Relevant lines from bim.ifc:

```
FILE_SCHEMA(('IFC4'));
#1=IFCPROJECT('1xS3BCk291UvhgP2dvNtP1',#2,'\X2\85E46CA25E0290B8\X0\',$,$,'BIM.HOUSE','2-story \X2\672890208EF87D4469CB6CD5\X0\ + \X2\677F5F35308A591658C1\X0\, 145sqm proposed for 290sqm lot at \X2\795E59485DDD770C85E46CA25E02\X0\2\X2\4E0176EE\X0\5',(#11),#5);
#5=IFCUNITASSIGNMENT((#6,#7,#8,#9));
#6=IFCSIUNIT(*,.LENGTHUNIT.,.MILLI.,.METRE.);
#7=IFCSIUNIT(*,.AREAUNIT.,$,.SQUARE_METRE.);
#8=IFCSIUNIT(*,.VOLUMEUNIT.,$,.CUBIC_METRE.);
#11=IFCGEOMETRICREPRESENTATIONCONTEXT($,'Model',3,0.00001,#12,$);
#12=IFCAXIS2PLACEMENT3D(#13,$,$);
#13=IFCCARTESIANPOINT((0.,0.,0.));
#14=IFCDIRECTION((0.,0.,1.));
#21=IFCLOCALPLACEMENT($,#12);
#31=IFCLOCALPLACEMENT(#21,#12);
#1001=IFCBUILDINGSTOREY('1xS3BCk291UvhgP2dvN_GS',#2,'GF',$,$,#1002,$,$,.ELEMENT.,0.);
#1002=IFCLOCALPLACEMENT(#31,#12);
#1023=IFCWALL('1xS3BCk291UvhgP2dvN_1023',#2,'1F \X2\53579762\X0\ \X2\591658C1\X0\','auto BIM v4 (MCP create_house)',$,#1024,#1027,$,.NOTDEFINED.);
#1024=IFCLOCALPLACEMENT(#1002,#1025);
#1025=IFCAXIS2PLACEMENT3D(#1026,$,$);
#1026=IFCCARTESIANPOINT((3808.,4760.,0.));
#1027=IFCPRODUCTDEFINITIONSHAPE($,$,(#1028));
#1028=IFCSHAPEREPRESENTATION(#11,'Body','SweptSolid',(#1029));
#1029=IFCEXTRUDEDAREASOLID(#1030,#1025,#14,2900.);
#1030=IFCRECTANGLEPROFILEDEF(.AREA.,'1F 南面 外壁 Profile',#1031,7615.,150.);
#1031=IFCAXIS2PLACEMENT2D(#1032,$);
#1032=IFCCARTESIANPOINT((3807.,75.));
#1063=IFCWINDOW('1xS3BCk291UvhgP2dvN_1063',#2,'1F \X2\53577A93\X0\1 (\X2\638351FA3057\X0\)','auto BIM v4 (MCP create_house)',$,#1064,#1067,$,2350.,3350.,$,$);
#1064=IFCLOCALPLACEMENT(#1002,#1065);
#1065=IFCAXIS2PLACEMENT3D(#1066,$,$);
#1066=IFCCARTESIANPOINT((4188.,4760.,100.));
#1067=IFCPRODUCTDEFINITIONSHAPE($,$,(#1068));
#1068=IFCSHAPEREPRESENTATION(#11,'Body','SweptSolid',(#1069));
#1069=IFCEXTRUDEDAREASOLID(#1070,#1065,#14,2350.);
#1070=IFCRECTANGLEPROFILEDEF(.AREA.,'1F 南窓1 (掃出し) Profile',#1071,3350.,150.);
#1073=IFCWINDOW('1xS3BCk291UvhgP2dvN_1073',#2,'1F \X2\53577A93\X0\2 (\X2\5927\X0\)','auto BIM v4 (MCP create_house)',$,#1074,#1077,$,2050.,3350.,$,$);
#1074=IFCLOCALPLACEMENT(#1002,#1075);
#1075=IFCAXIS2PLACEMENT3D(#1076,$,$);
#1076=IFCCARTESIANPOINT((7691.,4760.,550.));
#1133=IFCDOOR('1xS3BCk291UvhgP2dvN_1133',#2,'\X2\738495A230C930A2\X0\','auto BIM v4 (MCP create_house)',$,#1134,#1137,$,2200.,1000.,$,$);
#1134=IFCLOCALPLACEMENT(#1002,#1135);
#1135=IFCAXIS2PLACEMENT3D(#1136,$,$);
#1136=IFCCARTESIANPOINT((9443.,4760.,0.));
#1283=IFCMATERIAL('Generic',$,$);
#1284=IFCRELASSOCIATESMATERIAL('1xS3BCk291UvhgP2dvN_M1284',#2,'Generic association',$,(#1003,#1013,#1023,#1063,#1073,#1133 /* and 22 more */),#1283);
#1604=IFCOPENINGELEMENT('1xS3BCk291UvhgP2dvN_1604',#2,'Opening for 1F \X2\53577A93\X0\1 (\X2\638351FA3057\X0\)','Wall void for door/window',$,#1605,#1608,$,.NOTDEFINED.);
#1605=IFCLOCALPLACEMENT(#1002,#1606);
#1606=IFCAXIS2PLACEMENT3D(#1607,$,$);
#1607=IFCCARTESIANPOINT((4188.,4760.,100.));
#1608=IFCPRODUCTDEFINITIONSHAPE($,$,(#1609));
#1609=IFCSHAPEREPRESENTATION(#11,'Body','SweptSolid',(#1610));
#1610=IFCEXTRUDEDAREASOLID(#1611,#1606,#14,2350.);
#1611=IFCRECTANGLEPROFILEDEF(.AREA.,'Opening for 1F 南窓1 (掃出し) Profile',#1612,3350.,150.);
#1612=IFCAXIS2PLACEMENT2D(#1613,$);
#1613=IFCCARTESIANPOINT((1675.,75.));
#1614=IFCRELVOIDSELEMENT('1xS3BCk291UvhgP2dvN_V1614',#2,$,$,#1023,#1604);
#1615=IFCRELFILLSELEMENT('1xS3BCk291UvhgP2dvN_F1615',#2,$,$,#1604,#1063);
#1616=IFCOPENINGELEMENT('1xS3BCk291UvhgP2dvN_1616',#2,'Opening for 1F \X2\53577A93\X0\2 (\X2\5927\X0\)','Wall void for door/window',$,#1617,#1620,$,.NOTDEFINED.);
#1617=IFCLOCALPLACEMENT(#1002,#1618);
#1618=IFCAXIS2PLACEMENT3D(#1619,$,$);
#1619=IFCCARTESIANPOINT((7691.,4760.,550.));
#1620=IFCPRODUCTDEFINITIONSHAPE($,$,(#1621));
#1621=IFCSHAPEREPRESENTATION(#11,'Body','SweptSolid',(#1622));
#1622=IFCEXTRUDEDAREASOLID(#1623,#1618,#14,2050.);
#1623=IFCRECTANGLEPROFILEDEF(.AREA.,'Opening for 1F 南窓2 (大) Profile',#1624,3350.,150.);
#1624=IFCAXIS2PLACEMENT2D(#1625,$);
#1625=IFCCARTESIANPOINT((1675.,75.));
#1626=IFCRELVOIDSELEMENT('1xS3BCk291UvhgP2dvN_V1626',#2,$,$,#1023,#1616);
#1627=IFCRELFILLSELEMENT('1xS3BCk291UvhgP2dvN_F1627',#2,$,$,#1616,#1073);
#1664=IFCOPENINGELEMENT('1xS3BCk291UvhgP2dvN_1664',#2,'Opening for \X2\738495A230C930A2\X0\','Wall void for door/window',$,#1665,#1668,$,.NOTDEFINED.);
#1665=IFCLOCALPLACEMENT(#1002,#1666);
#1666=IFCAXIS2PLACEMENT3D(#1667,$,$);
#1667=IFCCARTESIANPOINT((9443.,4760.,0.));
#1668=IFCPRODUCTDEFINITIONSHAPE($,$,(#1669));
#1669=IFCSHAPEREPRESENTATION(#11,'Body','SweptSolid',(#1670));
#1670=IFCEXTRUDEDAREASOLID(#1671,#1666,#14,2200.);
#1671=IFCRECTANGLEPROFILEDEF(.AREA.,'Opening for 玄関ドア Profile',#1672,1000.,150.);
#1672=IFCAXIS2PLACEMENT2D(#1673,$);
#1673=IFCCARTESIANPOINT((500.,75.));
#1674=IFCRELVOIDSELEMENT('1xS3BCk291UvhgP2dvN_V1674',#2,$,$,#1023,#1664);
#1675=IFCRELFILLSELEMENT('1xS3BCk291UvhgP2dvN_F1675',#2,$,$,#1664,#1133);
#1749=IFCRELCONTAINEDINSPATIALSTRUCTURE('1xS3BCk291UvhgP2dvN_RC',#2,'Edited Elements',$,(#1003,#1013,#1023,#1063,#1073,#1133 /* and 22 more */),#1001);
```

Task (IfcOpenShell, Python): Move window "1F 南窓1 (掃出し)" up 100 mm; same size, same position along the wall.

```python
import numpy as np
import ifcopenshell
import ifcopenshell.api.geometry
import ifcopenshell.util.placement
import ifcopenshell.util.unit

model = ifcopenshell.open("bim.ifc")
unit_scale = ifcopenshell.util.unit.calculate_unit_scale(model)

window = model.by_guid("1xS3BCk291UvhgP2dvN_1063")
opening = window.FillsVoids[0].RelatingOpeningElement
dz = 0.1 / unit_scale

shift = np.array([0.0, 0.0, dz])
# The window is not placed relative to its opening, so move both.
for product in (opening, window):
    matrix = ifcopenshell.util.placement.get_local_placement(product.ObjectPlacement)
    matrix[:3, 3] += shift
    ifcopenshell.api.geometry.edit_object_placement(model, product=product, matrix=matrix, is_si=False)

print(f"moved by {dz * unit_scale:+.3f} m")

model.write("bim_v2.ifc")
```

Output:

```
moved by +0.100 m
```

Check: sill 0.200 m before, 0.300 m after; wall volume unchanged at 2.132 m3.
